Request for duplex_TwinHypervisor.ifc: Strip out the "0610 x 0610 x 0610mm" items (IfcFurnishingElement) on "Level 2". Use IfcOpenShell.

First a look at what the model holds.

```python
import ifcopenshell
import ifcopenshell.util.element

model = ifcopenshell.open("duplex_TwinHypervisor.ifc")
print(model.schema)
storey = next(s for s in model.by_type("IfcBuildingStorey") if s.Name == "Level 2")
furniture = [e for e in ifcopenshell.util.element.get_decomposition(storey) if e.is_a("IfcFurnishingElement")]
seen = {}
for e in furniture:
    element_type = ifcopenshell.util.element.get_type(e)
    name = element_type.Name if element_type not in (None, e) else None
    seen[name] = seen.get(name, 0) + 1
for name, count in sorted(seen.items(), key=str):
    print(count, "x", name)
```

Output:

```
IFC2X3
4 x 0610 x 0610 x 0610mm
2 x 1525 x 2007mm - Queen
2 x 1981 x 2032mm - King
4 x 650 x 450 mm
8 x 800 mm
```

```python
import ifcopenshell
import ifcopenshell.api.root
import ifcopenshell.util.element

model = ifcopenshell.open("duplex_TwinHypervisor.ifc")

storey = next(s for s in model.by_type("IfcBuildingStorey") if s.Name == "Level 2")
furniture = [e for e in ifcopenshell.util.element.get_decomposition(storey) if e.is_a("IfcFurnishingElement")]
targets = [e for e in furniture if (t := ifcopenshell.util.element.get_type(e)) not in (None, e) and t.Name == "0610 x 0610 x 0610mm"]

for e in targets:
    ifcopenshell.api.root.remove_product(model, product=e)
print(len(targets), "removed")

model.write("duplex_TwinHypervisor_rev.ifc")
```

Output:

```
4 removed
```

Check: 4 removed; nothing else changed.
